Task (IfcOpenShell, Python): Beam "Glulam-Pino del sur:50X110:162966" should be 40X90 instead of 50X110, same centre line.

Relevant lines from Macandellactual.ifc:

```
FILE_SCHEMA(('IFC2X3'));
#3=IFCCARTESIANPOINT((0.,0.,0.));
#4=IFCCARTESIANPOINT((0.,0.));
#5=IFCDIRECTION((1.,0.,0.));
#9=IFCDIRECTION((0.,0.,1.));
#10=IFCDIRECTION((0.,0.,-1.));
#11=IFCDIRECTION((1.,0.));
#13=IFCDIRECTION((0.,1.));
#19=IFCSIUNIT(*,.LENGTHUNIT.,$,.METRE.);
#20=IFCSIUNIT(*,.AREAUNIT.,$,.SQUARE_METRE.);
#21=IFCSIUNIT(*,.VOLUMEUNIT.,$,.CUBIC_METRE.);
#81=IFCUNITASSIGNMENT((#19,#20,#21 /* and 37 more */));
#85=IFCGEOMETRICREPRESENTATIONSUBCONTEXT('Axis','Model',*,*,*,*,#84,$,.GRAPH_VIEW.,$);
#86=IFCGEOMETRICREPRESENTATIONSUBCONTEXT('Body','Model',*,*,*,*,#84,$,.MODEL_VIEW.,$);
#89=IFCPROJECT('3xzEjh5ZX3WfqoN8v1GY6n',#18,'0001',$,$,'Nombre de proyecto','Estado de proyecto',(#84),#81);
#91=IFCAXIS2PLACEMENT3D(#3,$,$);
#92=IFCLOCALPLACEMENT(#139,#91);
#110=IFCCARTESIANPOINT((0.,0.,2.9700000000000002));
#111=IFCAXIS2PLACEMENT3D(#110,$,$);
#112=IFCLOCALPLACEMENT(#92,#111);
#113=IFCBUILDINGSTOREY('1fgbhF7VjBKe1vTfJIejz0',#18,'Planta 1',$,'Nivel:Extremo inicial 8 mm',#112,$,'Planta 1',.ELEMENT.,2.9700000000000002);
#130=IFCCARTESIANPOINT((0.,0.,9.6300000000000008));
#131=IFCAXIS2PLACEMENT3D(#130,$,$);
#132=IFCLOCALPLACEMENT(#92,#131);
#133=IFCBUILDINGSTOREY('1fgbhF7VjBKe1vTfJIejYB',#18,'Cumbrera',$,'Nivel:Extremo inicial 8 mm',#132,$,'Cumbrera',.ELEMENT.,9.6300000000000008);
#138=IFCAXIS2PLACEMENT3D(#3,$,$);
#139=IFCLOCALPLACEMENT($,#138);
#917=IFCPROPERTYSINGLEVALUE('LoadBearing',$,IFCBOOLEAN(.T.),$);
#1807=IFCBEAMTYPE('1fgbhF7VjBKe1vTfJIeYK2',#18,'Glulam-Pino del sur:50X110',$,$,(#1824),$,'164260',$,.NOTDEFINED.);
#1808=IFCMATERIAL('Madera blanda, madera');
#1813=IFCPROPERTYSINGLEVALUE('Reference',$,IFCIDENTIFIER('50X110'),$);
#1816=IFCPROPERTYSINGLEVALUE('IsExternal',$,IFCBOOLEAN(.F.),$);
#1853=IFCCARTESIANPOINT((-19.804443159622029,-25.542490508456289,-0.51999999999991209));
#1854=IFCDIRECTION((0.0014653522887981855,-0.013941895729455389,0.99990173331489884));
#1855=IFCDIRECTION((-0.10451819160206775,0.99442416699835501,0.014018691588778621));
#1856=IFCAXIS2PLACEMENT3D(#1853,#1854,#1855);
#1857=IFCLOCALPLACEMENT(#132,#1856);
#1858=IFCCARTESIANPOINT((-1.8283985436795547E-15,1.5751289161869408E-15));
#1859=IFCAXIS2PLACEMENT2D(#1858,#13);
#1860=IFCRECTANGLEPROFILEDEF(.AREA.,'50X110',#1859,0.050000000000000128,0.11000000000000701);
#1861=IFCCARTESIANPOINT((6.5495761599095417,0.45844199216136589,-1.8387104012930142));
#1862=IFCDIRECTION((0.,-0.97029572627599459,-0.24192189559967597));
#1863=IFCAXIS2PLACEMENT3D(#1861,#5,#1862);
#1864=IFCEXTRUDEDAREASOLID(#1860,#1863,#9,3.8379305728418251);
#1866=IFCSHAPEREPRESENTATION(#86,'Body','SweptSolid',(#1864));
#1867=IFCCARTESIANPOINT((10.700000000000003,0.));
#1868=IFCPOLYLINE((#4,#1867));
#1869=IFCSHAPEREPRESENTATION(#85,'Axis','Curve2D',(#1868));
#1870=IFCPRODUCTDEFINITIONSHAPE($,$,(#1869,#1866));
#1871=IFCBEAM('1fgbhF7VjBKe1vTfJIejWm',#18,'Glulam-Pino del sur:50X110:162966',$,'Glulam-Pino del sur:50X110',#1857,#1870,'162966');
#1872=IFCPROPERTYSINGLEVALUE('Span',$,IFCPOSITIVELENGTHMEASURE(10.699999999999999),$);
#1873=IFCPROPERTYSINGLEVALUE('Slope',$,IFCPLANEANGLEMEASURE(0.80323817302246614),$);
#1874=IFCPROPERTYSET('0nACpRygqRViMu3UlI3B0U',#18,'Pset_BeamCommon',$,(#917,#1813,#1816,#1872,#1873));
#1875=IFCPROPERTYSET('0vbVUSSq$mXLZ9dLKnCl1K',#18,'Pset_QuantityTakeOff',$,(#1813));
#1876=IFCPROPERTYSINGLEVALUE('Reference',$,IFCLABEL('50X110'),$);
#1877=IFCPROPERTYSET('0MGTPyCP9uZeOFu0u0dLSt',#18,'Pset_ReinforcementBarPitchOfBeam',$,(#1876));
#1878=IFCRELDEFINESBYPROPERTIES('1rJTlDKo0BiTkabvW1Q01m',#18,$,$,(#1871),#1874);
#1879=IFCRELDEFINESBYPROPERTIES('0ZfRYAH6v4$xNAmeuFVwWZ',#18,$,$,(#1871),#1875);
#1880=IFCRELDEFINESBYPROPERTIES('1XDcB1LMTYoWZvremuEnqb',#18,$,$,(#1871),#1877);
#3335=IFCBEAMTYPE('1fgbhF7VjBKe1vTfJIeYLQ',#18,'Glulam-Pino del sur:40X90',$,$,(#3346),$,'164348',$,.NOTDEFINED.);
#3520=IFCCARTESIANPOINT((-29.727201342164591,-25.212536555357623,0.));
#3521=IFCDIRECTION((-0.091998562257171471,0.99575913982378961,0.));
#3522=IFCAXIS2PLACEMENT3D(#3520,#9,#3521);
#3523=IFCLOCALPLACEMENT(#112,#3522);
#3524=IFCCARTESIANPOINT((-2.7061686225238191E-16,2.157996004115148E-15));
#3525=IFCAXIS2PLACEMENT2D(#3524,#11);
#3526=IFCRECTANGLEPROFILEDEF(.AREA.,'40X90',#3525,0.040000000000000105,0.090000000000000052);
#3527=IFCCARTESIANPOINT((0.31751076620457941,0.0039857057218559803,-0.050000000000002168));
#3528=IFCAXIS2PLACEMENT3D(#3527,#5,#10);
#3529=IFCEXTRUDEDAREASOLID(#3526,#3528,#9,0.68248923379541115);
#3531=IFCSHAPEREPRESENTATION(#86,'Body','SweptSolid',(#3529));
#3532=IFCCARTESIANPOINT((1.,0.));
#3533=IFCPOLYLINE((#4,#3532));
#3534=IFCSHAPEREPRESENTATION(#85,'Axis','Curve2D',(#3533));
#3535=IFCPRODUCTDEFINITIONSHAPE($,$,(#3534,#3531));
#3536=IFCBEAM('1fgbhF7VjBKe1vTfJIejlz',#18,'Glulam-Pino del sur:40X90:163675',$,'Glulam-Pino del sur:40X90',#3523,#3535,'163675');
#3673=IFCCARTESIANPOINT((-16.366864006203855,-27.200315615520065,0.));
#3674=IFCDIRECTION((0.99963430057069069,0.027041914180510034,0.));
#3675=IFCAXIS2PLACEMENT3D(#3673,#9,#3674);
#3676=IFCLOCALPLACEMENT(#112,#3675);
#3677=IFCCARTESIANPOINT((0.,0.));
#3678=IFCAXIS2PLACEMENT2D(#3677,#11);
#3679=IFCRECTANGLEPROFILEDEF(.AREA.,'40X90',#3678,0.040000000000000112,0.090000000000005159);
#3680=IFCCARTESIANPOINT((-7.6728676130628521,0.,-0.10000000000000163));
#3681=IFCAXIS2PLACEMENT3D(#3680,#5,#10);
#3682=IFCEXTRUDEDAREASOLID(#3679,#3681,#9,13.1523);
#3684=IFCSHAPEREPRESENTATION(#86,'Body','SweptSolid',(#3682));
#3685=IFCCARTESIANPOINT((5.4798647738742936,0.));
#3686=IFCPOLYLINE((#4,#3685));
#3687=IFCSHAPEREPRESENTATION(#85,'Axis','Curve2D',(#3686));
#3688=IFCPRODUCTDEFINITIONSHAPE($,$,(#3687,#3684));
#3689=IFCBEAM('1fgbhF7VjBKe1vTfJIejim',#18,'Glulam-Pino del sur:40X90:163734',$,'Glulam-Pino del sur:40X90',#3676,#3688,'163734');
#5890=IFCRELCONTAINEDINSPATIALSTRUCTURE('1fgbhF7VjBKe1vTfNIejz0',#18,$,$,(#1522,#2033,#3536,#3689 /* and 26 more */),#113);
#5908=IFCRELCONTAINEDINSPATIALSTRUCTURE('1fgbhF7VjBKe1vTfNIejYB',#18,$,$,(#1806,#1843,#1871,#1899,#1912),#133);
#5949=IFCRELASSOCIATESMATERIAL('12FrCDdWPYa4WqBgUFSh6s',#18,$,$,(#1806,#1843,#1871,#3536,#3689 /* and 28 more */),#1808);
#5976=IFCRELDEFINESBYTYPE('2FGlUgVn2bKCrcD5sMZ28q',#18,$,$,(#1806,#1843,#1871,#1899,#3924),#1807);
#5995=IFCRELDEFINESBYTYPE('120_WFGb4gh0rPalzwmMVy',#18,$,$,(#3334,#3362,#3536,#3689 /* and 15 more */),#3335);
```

```python
import ifcopenshell
import ifcopenshell.api.pset
import ifcopenshell.api.type
import ifcopenshell.util.element
import ifcopenshell.util.representation

model = ifcopenshell.open("Macandellactual.ifc")

member = model.by_id(1871)
source = next(p for p in model.by_type("IfcRectangleProfileDef") if p.ProfileName == "40X90")

body = ifcopenshell.util.representation.get_representation(member, "Model", "Body")
solid = body.Items[0]
old_profile = solid.SweptArea

# Copy the section's sizes but keep this member's own profile position.
profile = ifcopenshell.util.element.copy(model, source)
profile.Position = old_profile.Position
solid.SweptArea = profile
if not model.get_total_inverses(old_profile):
    ifcopenshell.util.element.remove_deep2(model, old_profile)

new_type = model.by_guid("1fgbhF7VjBKe1vTfJIeYLQ")
ifcopenshell.api.type.assign_type(
    model, related_objects=[member], relating_type=new_type, should_map_representations=False
)
member.Name = member.Name.replace("50X110", "40X90")
member.ObjectType = "Glulam-Pino del sur:40X90"
pset = model.by_id(ifcopenshell.util.element.get_pset(member, "Pset_BeamCommon", should_inherit=False)["id"])
ifcopenshell.api.pset.edit_pset(model, pset=pset, properties={"Reference": "40X90"})
pset = model.by_id(ifcopenshell.util.element.get_pset(member, "Pset_QuantityTakeOff", should_inherit=False)["id"])
ifcopenshell.api.pset.edit_pset(model, pset=pset, properties={"Reference": "40X90"})
pset = model.by_id(ifcopenshell.util.element.get_pset(member, "Pset_ReinforcementBarPitchOfBeam", should_inherit=False)["id"])
ifcopenshell.api.pset.edit_pset(model, pset=pset, properties={"Reference": "40X90"})

print(solid.SweptArea)

model.write("Macandellactual_v2.ifc")
```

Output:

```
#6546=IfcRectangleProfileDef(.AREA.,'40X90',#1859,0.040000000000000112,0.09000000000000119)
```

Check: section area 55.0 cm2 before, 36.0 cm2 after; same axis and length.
